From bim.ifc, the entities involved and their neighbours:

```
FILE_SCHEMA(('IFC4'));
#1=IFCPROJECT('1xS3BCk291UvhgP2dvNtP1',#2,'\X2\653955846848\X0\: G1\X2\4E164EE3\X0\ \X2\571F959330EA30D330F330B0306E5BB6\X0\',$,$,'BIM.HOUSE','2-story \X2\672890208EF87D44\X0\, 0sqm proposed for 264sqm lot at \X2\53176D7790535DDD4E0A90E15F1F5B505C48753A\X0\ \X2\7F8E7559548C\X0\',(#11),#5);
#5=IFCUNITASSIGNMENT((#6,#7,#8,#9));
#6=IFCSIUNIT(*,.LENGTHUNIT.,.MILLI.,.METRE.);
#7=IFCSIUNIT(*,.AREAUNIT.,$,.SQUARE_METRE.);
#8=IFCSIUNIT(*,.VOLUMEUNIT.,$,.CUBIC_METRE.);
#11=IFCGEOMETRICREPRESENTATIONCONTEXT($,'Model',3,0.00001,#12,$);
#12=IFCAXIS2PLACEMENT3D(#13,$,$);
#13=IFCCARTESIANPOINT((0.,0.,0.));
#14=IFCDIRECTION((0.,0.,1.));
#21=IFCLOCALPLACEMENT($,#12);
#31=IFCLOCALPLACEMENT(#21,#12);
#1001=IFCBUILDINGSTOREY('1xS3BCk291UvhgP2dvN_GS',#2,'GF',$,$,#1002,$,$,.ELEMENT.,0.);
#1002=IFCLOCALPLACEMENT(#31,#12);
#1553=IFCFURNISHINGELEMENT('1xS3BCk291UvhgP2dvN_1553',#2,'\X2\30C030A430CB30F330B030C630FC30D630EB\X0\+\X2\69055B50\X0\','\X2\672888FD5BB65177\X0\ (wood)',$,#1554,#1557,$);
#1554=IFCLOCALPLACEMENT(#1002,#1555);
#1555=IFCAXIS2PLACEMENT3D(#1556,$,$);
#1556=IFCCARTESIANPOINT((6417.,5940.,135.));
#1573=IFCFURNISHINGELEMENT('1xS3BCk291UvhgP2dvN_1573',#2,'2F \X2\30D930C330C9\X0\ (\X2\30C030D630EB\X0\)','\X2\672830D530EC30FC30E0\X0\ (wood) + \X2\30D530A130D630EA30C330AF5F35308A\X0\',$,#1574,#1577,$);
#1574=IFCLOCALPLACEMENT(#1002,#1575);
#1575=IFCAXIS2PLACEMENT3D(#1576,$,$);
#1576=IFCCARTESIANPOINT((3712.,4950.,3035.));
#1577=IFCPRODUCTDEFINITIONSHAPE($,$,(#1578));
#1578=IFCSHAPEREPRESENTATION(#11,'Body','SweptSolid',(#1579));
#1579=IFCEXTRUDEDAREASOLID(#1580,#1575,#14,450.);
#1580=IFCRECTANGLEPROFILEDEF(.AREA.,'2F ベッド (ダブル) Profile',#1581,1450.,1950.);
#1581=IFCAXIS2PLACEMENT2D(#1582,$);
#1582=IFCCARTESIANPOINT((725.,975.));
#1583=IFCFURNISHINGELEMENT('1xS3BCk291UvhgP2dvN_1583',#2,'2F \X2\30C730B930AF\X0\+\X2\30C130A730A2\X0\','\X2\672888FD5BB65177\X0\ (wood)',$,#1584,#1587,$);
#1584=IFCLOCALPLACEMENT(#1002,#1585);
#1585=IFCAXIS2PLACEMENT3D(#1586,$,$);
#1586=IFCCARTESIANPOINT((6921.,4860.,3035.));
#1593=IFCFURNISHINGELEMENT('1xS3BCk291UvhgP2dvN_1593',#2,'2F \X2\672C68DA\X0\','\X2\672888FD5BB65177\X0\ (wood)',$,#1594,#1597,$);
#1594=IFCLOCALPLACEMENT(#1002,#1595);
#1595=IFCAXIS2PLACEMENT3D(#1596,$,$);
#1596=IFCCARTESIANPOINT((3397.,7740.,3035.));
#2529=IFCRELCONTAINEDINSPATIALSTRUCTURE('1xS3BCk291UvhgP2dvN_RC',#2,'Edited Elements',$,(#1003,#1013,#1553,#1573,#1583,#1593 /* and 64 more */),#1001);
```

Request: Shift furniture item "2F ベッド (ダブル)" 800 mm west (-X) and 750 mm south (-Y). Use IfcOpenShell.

```python
import ifcopenshell
import ifcopenshell.api.geometry
import ifcopenshell.util.placement
import ifcopenshell.util.unit

model = ifcopenshell.open("bim.ifc")
unit_scale = ifcopenshell.util.unit.calculate_unit_scale(model)

item = model.by_guid("1xS3BCk291UvhgP2dvN_1573")
matrix = ifcopenshell.util.placement.get_local_placement(item.ObjectPlacement)
matrix[0, 3] -= 0.8 / unit_scale
matrix[1, 3] -= 0.75 / unit_scale
ifcopenshell.api.geometry.edit_object_placement(model, product=item, matrix=matrix, is_si=False)

print(ifcopenshell.util.placement.get_local_placement(item.ObjectPlacement).round(3) + 0.0)

model.write("bim-out.ifc")
```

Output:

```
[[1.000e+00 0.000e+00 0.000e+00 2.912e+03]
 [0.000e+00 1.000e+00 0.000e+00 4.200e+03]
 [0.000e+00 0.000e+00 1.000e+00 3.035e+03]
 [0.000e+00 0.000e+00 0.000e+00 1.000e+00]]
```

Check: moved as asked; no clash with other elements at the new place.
